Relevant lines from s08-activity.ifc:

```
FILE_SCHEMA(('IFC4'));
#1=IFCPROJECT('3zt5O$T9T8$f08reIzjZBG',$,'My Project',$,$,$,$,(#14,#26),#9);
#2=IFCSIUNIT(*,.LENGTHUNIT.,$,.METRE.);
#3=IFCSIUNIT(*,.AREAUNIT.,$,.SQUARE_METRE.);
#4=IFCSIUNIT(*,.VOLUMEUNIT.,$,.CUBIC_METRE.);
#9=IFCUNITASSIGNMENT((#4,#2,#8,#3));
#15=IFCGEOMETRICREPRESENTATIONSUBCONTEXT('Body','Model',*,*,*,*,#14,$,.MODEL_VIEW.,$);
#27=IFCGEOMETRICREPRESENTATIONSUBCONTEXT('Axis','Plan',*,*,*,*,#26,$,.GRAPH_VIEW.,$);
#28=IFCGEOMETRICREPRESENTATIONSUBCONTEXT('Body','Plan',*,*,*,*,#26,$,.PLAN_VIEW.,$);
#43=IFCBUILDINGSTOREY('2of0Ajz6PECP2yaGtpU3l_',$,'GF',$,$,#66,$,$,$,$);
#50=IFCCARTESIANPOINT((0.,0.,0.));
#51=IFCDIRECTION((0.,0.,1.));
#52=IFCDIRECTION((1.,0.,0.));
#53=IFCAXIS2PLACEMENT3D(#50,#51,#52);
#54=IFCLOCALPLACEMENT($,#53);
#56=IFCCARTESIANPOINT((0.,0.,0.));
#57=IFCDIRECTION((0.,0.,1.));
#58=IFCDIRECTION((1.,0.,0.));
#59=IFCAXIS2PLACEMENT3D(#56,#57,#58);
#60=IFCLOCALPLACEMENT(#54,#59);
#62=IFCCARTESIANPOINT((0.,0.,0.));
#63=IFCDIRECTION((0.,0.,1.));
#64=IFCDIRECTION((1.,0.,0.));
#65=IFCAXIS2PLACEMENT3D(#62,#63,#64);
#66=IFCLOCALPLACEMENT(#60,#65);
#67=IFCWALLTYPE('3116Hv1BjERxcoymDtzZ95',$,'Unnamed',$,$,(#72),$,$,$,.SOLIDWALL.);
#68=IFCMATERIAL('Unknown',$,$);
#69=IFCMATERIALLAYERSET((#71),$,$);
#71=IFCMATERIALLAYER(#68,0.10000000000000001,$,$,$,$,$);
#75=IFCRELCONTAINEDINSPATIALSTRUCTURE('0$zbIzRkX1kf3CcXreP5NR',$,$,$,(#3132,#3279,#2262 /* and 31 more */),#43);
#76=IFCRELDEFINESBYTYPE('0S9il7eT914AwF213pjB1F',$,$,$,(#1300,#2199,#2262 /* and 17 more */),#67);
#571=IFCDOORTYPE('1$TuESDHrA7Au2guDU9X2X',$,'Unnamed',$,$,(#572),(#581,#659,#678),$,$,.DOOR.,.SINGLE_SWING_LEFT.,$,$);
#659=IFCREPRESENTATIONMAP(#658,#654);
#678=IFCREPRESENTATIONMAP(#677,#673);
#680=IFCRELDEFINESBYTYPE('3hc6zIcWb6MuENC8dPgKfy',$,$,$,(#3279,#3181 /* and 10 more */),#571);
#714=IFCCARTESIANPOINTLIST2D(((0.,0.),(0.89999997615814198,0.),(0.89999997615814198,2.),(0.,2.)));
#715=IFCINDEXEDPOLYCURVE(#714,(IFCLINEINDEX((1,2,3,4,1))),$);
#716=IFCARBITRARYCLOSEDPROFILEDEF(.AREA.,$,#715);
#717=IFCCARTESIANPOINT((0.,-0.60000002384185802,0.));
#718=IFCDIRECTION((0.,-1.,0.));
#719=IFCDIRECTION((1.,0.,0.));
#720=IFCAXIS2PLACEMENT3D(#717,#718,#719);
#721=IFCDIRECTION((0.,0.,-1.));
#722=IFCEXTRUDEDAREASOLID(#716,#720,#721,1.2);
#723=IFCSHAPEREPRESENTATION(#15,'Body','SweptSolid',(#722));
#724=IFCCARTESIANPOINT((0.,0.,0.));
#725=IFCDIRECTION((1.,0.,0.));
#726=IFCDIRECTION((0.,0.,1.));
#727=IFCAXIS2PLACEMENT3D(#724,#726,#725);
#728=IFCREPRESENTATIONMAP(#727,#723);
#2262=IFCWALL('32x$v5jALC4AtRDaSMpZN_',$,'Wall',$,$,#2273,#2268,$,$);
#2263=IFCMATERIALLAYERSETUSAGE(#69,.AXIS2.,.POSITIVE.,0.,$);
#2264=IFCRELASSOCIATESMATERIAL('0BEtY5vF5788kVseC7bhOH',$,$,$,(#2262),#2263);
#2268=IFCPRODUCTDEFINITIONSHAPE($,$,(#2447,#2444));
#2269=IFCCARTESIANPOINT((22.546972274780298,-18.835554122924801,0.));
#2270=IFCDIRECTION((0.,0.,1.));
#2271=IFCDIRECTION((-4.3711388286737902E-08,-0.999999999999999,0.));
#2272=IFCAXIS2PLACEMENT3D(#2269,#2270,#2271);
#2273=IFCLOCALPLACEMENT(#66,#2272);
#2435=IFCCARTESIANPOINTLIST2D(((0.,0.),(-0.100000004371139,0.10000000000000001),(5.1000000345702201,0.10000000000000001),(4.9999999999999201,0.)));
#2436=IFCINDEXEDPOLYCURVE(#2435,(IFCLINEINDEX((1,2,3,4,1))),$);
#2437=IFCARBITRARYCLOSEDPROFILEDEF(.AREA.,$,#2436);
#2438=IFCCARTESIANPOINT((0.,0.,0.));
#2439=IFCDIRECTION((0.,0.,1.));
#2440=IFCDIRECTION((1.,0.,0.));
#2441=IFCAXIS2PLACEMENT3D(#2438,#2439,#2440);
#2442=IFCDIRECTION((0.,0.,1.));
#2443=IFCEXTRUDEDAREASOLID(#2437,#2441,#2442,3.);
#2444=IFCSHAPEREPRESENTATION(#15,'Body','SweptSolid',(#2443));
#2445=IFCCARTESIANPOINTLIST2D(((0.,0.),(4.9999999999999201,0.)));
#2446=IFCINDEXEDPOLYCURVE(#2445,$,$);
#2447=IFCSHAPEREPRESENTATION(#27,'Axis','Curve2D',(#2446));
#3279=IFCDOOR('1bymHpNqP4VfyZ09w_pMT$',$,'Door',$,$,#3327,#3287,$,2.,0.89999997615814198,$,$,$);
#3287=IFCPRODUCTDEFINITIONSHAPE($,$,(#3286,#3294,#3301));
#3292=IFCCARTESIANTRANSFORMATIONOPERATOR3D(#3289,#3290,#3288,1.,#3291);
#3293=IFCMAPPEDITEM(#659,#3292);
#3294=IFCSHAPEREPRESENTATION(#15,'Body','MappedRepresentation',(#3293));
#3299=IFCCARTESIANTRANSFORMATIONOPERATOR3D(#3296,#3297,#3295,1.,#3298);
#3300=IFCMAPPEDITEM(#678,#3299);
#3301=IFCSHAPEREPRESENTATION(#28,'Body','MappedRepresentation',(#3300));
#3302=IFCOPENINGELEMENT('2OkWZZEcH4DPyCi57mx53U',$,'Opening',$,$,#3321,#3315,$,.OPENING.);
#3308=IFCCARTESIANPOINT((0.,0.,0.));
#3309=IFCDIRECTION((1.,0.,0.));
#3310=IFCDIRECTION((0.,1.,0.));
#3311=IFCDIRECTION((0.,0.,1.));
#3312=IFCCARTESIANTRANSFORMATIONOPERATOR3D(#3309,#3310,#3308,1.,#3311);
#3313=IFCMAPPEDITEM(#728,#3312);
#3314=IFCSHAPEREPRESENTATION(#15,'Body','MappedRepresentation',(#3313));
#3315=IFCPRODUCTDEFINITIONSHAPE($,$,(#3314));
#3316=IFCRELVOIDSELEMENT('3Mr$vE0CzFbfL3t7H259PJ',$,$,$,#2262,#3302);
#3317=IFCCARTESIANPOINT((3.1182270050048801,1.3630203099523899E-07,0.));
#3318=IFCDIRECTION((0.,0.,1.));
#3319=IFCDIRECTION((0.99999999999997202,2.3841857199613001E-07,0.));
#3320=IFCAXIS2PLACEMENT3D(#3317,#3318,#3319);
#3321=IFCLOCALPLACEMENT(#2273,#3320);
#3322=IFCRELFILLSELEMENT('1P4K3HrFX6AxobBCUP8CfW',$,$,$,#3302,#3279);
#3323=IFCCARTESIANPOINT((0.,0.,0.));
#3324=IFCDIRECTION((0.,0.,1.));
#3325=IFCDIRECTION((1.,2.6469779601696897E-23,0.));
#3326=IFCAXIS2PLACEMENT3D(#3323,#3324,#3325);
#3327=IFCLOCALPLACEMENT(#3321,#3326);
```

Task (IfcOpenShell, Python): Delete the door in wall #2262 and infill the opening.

```python
import ifcopenshell
import ifcopenshell.api.feature
import ifcopenshell.api.root
import ifcopenshell.geom
import ifcopenshell.util.shape

model = ifcopenshell.open("s08-activity.ifc")
settings = ifcopenshell.geom.settings()


def volume(element):
    """Net volume in cubic metres, openings subtracted."""
    shape = ifcopenshell.geom.create_shape(settings, element)
    return ifcopenshell.util.shape.get_volume(shape.geometry)


door = model.by_guid("1bymHpNqP4VfyZ09w_pMT$")
opening = door.FillsVoids[0].RelatingOpeningElement
wall = opening.VoidsElements[0].RelatingBuildingElement
before = volume(wall)

ifcopenshell.api.root.remove_product(model, product=door)
ifcopenshell.api.feature.remove_feature(model, feature=opening)

after = volume(wall)

print(f"wall volume {before:.3f} -> {after:.3f} m3")

model.write("s08-activity_updated.ifc")
```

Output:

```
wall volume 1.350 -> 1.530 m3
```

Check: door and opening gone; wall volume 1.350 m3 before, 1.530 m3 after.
